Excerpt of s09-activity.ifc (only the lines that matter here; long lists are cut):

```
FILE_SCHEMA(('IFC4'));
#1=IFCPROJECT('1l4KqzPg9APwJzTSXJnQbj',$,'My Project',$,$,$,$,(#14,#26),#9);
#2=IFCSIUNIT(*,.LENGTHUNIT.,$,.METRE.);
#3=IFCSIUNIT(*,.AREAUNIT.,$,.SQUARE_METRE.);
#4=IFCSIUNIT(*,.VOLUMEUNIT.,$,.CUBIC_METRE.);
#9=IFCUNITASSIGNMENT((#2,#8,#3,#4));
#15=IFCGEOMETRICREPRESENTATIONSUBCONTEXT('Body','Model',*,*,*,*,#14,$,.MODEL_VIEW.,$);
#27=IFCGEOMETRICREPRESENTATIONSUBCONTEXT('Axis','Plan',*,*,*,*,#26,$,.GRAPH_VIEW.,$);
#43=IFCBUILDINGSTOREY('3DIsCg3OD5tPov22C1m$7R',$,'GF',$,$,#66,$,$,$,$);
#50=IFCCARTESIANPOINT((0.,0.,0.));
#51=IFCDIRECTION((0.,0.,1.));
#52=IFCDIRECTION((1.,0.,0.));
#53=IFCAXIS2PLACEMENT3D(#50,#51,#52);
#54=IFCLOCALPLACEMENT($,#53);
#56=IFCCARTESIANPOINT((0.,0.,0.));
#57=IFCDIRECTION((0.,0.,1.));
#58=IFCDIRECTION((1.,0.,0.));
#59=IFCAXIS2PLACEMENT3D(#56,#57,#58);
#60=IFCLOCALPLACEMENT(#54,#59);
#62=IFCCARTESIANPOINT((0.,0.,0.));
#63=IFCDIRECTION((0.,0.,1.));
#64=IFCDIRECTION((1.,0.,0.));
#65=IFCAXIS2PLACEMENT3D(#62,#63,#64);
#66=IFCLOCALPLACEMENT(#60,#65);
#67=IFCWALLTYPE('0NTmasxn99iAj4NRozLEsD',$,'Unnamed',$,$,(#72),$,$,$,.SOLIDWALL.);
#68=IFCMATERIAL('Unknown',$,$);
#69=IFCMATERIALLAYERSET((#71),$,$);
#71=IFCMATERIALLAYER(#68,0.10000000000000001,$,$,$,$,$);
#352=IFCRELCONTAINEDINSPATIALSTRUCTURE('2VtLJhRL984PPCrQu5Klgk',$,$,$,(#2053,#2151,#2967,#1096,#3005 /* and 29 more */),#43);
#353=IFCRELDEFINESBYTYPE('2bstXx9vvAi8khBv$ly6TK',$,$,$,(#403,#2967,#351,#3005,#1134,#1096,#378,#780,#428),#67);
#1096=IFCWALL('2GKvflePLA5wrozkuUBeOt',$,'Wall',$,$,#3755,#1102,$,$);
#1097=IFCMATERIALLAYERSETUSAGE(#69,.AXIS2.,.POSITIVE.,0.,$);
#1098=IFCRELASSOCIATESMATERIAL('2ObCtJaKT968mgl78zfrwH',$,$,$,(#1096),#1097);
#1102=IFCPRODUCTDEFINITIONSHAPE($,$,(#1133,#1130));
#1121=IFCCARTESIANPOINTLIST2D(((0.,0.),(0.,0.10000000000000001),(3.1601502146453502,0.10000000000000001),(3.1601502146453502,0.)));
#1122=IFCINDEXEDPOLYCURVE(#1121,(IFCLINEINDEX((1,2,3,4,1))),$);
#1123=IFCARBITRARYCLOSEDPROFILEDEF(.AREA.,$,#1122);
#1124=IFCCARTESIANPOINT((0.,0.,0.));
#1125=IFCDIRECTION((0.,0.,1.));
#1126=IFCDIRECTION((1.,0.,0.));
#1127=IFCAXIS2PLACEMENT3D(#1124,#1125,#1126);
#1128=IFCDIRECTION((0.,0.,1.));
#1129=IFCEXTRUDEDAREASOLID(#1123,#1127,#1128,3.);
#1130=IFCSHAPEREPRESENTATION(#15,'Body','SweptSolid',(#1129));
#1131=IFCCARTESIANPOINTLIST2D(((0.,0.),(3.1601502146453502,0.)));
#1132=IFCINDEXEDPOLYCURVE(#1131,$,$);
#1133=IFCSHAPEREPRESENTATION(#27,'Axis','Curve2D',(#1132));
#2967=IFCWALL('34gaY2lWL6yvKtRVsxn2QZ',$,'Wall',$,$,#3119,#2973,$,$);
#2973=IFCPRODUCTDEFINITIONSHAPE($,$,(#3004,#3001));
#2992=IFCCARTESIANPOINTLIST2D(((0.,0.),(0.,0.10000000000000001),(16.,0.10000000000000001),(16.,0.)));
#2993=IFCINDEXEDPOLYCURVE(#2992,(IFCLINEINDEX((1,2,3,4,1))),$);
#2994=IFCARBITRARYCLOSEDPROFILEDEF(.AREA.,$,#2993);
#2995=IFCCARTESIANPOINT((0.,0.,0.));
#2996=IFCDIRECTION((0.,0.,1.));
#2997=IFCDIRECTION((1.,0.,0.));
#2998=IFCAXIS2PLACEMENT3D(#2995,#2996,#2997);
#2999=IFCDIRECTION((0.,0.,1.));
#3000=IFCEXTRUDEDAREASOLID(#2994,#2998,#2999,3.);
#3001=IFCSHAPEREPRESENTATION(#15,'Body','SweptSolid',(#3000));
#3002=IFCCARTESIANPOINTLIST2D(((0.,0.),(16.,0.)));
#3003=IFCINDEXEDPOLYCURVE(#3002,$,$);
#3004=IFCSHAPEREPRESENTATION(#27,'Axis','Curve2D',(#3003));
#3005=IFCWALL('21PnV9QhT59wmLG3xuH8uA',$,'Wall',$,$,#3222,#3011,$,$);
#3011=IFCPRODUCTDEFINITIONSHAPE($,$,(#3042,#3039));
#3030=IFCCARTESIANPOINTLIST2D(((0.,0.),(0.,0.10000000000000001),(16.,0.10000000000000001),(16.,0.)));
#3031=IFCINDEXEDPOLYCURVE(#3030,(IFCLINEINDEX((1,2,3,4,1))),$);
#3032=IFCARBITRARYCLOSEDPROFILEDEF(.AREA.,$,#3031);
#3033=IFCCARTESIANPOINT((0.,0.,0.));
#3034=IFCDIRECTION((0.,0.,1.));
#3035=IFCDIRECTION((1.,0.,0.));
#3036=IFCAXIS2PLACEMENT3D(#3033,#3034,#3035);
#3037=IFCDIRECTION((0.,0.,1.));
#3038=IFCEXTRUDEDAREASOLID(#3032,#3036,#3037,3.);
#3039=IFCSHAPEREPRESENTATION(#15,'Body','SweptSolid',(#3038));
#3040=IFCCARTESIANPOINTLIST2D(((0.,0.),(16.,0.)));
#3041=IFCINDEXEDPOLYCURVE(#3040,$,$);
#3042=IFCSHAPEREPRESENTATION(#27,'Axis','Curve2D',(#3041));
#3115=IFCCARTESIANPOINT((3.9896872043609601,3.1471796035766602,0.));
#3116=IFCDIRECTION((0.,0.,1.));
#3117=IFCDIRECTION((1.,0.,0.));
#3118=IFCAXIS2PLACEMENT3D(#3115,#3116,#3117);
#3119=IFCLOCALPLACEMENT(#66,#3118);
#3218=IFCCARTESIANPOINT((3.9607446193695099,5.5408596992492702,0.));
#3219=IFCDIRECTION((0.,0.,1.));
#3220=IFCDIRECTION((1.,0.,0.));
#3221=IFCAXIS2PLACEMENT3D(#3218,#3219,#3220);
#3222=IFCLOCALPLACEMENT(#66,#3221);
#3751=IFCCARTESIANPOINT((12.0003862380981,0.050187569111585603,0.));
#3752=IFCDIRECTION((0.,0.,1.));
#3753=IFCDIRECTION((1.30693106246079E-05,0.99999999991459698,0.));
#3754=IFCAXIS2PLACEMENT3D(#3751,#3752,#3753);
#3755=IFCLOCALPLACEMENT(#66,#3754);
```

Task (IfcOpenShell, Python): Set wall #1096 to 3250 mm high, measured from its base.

```python
import ifcopenshell
import ifcopenshell.geom
import ifcopenshell.util.representation
import ifcopenshell.util.shape
import ifcopenshell.util.unit

model = ifcopenshell.open("s09-activity.ifc")
unit_scale = ifcopenshell.util.unit.calculate_unit_scale(model)
settings = ifcopenshell.geom.settings()


def volume(element):
    """Net volume in cubic metres, openings subtracted."""
    shape = ifcopenshell.geom.create_shape(settings, element)
    return ifcopenshell.util.shape.get_volume(shape.geometry)


wall = model.by_guid("2GKvflePLA5wrozkuUBeOt")
before = volume(wall)

body = ifcopenshell.util.representation.get_representation(wall, "Model", "Body")
solid = body.Items[0]
old_height = solid.Depth
solid.Depth = 3.25 / unit_scale
after = volume(wall)

print(f"height {old_height:g} -> {solid.Depth:g}, volume {before:.3f} -> {after:.3f} m3")

model.write("s09-activity_v2.ifc")
```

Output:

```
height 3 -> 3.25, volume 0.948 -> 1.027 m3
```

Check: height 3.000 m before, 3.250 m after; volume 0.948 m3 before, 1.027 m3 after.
